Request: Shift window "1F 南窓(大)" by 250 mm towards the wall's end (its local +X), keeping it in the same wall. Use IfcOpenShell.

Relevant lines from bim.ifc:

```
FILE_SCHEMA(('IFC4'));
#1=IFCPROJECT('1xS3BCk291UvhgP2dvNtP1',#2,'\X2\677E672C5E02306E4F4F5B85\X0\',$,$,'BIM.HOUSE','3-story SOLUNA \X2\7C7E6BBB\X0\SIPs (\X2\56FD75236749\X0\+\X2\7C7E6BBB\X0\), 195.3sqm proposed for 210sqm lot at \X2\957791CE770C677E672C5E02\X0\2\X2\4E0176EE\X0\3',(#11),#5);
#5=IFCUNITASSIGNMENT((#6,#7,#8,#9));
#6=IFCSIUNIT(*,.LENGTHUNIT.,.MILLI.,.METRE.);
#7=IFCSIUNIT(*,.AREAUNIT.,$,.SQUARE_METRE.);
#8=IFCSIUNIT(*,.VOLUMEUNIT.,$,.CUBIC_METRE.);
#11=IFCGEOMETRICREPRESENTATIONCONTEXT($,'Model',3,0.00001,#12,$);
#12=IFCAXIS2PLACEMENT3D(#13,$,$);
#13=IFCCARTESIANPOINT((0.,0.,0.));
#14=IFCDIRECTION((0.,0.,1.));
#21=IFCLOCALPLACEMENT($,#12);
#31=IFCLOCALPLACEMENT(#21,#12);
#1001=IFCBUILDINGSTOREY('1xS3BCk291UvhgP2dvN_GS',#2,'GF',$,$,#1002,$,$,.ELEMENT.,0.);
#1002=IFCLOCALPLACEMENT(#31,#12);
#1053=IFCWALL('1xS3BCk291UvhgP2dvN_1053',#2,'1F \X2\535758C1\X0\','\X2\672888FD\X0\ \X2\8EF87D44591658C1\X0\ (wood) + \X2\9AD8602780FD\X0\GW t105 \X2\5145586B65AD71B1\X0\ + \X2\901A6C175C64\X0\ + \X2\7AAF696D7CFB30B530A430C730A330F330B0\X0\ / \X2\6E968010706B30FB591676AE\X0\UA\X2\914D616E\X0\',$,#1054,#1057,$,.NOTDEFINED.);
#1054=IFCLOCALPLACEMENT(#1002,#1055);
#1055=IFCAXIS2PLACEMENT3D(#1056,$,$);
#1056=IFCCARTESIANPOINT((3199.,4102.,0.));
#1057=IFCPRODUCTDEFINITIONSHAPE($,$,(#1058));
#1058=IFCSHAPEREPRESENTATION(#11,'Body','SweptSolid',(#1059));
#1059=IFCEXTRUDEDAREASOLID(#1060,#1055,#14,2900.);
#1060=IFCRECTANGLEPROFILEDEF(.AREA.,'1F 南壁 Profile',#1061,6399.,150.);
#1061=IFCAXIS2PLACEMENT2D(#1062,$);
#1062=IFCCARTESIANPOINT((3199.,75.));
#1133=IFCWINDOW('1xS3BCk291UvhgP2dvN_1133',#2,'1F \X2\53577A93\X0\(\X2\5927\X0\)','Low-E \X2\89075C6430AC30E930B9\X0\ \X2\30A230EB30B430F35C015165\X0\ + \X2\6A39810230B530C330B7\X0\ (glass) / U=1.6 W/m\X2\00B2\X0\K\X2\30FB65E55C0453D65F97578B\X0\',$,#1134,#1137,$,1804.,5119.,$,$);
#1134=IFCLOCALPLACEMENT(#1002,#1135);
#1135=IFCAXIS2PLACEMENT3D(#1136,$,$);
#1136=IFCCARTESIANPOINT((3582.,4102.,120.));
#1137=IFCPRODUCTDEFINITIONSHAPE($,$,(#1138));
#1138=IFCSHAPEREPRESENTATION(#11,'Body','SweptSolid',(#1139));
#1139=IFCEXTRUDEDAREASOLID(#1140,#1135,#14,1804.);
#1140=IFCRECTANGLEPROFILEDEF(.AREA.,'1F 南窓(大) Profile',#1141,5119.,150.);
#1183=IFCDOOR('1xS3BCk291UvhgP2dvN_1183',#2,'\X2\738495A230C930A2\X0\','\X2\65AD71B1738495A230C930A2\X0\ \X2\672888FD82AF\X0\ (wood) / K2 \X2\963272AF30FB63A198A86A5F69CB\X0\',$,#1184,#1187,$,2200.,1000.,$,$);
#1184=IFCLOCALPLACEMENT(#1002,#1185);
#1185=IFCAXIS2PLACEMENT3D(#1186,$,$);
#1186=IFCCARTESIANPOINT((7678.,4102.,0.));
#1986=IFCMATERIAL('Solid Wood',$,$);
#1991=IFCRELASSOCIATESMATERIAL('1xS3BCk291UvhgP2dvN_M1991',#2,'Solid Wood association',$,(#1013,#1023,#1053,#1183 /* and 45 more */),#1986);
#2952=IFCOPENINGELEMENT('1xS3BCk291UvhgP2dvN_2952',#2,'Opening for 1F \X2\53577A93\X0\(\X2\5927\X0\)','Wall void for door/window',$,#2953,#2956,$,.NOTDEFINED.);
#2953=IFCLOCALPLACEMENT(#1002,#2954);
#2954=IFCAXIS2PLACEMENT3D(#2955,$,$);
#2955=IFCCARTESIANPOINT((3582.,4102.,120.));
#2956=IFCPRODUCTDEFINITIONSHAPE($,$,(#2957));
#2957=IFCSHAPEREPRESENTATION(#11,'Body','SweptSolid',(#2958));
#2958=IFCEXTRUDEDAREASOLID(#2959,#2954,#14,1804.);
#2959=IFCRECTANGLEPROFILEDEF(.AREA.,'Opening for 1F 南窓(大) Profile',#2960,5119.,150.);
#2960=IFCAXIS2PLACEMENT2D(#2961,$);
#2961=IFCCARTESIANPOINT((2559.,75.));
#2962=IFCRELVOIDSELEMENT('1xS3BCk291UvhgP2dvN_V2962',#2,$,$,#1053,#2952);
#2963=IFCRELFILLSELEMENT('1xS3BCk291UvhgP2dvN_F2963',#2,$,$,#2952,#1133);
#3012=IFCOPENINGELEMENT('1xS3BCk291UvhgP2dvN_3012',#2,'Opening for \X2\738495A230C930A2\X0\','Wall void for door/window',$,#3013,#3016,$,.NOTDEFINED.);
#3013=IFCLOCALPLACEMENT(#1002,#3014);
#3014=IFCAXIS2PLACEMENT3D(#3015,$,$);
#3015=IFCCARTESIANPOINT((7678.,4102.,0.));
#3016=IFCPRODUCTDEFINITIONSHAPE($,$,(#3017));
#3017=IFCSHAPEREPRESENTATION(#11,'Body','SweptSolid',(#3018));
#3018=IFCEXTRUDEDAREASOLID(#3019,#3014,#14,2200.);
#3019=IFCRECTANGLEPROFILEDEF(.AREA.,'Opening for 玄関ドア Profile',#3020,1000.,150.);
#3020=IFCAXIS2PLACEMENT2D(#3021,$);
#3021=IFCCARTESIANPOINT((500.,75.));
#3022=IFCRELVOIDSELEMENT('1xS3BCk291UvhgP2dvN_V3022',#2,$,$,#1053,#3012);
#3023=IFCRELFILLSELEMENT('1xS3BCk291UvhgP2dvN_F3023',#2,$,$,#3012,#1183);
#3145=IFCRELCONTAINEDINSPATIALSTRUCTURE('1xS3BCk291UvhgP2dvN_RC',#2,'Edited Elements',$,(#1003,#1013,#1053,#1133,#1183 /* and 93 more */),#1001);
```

```python
import ifcopenshell
import ifcopenshell.api.geometry
import ifcopenshell.util.placement
import ifcopenshell.util.unit

model = ifcopenshell.open("bim.ifc")
unit_scale = ifcopenshell.util.unit.calculate_unit_scale(model)

window = model.by_guid("1xS3BCk291UvhgP2dvN_1133")
opening = window.FillsVoids[0].RelatingOpeningElement
wall = opening.VoidsElements[0].RelatingBuildingElement

wall_matrix = ifcopenshell.util.placement.get_local_placement(wall.ObjectPlacement)
shift = wall_matrix[:3, 0] * 0.25 / unit_scale
before = ifcopenshell.util.placement.get_local_placement(window.ObjectPlacement)[:3, 3].copy()

# The window is not placed relative to its opening, so move both.
for product in (opening, window):
    matrix = ifcopenshell.util.placement.get_local_placement(product.ObjectPlacement)
    matrix[:3, 3] += shift
    ifcopenshell.api.geometry.edit_object_placement(model, product=product, matrix=matrix, is_si=False)

after = ifcopenshell.util.placement.get_local_placement(window.ObjectPlacement)[:3, 3]
print("window moved by", (after - before).round(3) + 0.0)

model.write("bim-out.ifc")
```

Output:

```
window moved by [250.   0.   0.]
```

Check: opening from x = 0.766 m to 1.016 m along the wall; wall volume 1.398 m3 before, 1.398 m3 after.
